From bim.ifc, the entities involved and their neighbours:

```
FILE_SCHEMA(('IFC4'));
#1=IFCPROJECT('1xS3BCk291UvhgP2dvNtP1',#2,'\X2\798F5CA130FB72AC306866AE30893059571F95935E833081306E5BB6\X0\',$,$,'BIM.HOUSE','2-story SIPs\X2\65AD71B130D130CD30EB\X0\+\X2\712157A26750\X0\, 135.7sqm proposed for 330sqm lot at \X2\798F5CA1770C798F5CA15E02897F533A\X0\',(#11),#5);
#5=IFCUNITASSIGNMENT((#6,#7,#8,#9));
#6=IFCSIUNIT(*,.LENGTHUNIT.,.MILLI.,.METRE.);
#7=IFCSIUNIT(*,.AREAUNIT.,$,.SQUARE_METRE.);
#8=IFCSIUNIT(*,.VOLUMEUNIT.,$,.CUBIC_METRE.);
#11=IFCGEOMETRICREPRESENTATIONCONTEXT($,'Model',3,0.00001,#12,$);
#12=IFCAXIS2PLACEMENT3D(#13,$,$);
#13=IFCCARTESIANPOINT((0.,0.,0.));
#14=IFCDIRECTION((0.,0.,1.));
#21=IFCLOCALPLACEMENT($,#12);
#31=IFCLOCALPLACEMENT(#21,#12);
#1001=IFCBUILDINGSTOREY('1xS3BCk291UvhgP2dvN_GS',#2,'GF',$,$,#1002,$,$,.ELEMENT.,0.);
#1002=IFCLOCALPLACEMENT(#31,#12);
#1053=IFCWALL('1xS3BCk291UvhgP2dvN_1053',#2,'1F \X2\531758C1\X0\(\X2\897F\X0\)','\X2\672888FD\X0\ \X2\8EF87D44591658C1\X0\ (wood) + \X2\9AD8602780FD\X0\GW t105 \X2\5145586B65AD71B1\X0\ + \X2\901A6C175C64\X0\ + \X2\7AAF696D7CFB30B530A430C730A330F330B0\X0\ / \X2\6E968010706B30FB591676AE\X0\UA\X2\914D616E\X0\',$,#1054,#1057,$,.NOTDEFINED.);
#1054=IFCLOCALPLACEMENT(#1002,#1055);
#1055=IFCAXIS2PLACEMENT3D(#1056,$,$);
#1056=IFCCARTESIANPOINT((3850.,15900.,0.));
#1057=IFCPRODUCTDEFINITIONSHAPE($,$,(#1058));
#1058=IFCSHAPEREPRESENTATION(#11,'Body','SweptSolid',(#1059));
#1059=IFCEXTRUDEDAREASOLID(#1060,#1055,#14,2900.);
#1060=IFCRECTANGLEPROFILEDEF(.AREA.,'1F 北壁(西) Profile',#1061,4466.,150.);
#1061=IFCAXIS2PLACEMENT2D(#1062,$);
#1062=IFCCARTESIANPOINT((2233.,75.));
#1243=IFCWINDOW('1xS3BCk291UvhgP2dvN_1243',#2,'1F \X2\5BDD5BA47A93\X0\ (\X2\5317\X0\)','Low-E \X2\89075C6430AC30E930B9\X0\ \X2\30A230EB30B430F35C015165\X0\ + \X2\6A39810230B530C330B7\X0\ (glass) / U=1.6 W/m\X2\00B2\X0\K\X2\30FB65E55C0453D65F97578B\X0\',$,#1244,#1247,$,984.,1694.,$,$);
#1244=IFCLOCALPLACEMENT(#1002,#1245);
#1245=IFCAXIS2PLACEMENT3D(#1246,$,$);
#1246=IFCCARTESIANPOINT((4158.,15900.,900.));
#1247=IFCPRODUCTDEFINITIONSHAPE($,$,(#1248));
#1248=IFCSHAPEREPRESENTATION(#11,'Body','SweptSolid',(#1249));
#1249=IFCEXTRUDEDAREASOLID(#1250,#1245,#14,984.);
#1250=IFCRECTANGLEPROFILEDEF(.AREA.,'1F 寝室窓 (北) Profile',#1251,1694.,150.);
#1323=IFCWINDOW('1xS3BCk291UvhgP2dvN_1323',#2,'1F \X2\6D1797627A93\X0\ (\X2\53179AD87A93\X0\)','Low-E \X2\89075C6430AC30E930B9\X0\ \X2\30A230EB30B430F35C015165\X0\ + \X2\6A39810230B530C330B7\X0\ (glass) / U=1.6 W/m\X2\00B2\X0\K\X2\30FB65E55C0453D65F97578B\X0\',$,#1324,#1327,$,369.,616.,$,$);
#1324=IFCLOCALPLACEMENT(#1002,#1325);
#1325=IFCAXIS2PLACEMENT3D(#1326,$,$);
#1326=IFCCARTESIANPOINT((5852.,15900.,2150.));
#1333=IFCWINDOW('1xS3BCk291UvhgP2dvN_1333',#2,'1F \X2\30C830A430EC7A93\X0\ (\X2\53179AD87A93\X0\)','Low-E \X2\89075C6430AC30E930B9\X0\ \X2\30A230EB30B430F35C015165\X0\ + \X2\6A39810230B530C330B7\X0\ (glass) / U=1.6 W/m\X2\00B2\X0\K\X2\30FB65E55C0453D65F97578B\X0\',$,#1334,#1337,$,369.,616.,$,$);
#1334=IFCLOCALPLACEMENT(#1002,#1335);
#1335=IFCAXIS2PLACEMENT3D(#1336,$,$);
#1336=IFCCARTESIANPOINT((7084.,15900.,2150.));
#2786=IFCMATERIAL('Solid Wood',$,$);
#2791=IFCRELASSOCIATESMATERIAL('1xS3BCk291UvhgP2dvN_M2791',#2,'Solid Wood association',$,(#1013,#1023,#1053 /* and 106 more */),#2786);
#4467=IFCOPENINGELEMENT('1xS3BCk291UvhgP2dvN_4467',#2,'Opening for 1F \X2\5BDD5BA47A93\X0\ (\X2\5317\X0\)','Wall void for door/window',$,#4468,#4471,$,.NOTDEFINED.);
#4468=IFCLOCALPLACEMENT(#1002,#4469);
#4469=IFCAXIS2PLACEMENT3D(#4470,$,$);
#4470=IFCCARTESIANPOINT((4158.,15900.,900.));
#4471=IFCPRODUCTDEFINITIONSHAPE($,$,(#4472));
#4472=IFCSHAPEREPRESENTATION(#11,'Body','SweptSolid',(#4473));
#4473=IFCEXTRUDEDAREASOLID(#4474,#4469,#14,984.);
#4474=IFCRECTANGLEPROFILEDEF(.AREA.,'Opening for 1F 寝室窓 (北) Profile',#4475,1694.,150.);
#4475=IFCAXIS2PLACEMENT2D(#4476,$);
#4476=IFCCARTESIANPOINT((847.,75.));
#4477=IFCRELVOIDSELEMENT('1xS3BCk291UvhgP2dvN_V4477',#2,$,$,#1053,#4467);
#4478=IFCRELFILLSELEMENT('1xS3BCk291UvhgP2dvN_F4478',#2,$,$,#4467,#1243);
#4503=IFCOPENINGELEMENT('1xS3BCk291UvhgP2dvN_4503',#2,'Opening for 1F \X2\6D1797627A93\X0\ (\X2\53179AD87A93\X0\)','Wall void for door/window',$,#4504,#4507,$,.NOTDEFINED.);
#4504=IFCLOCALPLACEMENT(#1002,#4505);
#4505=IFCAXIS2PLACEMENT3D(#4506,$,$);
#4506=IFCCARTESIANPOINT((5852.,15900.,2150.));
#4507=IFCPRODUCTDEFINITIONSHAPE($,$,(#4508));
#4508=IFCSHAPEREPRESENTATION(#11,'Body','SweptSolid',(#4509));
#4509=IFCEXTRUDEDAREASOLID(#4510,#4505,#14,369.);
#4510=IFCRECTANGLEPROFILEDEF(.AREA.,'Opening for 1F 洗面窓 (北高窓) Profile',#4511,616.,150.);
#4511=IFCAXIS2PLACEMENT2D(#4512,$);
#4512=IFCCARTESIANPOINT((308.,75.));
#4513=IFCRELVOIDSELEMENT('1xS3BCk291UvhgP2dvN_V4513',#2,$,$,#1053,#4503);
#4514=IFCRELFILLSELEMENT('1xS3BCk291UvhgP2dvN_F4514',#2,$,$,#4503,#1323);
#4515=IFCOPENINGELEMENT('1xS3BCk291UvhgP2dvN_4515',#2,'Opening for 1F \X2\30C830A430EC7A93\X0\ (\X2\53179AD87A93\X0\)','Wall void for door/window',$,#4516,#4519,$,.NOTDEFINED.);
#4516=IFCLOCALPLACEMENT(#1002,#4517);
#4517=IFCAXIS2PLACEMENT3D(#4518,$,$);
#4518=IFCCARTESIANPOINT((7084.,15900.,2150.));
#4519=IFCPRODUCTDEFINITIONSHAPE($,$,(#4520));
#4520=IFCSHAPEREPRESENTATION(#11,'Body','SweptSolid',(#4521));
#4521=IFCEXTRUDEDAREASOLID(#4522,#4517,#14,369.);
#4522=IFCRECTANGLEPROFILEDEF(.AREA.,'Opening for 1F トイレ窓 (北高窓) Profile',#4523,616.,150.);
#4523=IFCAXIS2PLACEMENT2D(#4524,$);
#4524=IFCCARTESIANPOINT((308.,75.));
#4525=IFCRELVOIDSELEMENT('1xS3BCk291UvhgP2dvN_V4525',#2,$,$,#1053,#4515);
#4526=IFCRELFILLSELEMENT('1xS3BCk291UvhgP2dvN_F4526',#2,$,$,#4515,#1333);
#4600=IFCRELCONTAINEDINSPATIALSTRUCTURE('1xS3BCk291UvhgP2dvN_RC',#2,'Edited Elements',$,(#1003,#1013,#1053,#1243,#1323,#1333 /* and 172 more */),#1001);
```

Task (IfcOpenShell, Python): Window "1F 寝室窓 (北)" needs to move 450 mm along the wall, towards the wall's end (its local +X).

```python
import ifcopenshell
import ifcopenshell.api.geometry
import ifcopenshell.util.placement
import ifcopenshell.util.unit

model = ifcopenshell.open("bim.ifc")
unit_scale = ifcopenshell.util.unit.calculate_unit_scale(model)

window = model.by_guid("1xS3BCk291UvhgP2dvN_1243")
opening = window.FillsVoids[0].RelatingOpeningElement
wall = opening.VoidsElements[0].RelatingBuildingElement

wall_matrix = ifcopenshell.util.placement.get_local_placement(wall.ObjectPlacement)
shift = wall_matrix[:3, 0] * 0.45 / unit_scale
before = ifcopenshell.util.placement.get_local_placement(window.ObjectPlacement)[:3, 3].copy()

# The window is not placed relative to its opening, so move both.
for product in (opening, window):
    matrix = ifcopenshell.util.placement.get_local_placement(product.ObjectPlacement)
    matrix[:3, 3] += shift
    ifcopenshell.api.geometry.edit_object_placement(model, product=product, matrix=matrix, is_si=False)

after = ifcopenshell.util.placement.get_local_placement(window.ObjectPlacement)[:3, 3]
print("window moved by", (after - before).round(3) + 0.0)

model.write("bim_v2.ifc")
```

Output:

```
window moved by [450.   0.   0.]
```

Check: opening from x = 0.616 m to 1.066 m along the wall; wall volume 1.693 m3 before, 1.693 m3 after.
